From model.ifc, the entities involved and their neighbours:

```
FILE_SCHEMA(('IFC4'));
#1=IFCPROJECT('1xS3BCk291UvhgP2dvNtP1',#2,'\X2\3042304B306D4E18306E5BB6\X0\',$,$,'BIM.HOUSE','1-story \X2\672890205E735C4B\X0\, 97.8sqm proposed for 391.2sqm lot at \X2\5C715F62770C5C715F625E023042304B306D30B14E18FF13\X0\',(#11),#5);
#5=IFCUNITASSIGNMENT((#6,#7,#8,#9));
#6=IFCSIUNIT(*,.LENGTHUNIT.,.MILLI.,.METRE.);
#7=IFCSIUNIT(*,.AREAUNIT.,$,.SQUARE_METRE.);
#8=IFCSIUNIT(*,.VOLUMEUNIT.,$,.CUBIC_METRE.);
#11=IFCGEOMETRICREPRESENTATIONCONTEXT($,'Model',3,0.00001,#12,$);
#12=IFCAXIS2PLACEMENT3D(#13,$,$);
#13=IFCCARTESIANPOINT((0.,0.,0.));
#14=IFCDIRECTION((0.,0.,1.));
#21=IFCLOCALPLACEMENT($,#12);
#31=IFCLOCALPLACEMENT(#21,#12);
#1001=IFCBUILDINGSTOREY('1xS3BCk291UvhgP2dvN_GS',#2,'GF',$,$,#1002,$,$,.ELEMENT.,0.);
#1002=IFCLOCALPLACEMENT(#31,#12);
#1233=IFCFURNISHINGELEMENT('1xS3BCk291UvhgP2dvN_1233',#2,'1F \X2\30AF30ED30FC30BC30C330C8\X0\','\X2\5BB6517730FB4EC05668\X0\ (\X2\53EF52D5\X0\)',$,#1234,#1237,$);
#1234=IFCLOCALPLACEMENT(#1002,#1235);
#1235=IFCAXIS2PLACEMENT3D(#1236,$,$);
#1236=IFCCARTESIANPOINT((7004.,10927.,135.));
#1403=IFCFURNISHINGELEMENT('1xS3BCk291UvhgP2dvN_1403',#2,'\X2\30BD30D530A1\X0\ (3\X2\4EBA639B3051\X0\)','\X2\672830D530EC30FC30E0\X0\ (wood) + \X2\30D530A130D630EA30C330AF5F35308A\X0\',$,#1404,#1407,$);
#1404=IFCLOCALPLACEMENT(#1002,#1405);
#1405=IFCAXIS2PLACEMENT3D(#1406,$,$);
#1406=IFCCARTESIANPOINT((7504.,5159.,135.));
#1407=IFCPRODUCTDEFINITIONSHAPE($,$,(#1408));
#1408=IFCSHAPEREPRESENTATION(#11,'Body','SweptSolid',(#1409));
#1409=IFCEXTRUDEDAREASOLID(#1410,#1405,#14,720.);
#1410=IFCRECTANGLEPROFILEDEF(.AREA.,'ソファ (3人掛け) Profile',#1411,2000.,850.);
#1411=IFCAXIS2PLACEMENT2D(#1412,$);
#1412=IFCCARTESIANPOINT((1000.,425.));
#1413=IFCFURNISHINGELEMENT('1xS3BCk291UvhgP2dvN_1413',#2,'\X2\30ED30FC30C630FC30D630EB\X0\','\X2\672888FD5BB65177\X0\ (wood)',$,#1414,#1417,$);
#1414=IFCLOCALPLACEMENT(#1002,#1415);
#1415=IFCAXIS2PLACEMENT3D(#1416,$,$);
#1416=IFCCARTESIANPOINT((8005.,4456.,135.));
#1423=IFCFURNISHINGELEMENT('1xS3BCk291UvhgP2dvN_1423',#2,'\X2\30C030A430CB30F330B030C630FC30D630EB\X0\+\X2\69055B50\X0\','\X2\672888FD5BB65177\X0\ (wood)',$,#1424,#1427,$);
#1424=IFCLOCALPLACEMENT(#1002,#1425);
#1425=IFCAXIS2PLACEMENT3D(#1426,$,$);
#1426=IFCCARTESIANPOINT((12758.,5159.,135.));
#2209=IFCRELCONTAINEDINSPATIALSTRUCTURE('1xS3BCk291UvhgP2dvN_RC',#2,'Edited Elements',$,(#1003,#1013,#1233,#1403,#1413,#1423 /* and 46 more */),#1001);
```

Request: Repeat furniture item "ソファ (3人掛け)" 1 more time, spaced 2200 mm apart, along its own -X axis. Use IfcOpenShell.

```python
import ifcopenshell
import ifcopenshell.api.geometry
import ifcopenshell.api.root
import ifcopenshell.util.element
import ifcopenshell.util.placement
import ifcopenshell.util.unit

model = ifcopenshell.open("model.ifc")
unit_scale = ifcopenshell.util.unit.calculate_unit_scale(model)


def reuse_history(source, copy):
    """copy_class also copies each property set's owner history, people and application; keep the originals."""
    for rel in copy.IsDefinedBy:
        if rel.is_a("IfcRelDefinesByProperties") and (history := rel.RelatingPropertyDefinition.OwnerHistory):
            rel.RelatingPropertyDefinition.OwnerHistory = source.OwnerHistory
            ifcopenshell.util.element.remove_deep2(model, history)


source = model.by_id(1403)
base = ifcopenshell.util.placement.get_local_placement(source.ObjectPlacement)
step = -base[:3, 0] * 2.2 / unit_scale

for i in range(1, 2):
    copy = ifcopenshell.api.root.copy_class(model, product=source)
    copy.Representation = ifcopenshell.util.element.copy_deep(
        model, source.Representation, exclude=["IfcGeometricRepresentationContext", "IfcRepresentationMap"]
    )
    reuse_history(source, copy)
    matrix = base.copy()
    matrix[:3, 3] += i * step
    print("added at", matrix[:3, 3].round(3) + 0.0)
    ifcopenshell.api.geometry.edit_object_placement(model, product=copy, matrix=matrix, is_si=False)

model.write("model_v2.ifc")
```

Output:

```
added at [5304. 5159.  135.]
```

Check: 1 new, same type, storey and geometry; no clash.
